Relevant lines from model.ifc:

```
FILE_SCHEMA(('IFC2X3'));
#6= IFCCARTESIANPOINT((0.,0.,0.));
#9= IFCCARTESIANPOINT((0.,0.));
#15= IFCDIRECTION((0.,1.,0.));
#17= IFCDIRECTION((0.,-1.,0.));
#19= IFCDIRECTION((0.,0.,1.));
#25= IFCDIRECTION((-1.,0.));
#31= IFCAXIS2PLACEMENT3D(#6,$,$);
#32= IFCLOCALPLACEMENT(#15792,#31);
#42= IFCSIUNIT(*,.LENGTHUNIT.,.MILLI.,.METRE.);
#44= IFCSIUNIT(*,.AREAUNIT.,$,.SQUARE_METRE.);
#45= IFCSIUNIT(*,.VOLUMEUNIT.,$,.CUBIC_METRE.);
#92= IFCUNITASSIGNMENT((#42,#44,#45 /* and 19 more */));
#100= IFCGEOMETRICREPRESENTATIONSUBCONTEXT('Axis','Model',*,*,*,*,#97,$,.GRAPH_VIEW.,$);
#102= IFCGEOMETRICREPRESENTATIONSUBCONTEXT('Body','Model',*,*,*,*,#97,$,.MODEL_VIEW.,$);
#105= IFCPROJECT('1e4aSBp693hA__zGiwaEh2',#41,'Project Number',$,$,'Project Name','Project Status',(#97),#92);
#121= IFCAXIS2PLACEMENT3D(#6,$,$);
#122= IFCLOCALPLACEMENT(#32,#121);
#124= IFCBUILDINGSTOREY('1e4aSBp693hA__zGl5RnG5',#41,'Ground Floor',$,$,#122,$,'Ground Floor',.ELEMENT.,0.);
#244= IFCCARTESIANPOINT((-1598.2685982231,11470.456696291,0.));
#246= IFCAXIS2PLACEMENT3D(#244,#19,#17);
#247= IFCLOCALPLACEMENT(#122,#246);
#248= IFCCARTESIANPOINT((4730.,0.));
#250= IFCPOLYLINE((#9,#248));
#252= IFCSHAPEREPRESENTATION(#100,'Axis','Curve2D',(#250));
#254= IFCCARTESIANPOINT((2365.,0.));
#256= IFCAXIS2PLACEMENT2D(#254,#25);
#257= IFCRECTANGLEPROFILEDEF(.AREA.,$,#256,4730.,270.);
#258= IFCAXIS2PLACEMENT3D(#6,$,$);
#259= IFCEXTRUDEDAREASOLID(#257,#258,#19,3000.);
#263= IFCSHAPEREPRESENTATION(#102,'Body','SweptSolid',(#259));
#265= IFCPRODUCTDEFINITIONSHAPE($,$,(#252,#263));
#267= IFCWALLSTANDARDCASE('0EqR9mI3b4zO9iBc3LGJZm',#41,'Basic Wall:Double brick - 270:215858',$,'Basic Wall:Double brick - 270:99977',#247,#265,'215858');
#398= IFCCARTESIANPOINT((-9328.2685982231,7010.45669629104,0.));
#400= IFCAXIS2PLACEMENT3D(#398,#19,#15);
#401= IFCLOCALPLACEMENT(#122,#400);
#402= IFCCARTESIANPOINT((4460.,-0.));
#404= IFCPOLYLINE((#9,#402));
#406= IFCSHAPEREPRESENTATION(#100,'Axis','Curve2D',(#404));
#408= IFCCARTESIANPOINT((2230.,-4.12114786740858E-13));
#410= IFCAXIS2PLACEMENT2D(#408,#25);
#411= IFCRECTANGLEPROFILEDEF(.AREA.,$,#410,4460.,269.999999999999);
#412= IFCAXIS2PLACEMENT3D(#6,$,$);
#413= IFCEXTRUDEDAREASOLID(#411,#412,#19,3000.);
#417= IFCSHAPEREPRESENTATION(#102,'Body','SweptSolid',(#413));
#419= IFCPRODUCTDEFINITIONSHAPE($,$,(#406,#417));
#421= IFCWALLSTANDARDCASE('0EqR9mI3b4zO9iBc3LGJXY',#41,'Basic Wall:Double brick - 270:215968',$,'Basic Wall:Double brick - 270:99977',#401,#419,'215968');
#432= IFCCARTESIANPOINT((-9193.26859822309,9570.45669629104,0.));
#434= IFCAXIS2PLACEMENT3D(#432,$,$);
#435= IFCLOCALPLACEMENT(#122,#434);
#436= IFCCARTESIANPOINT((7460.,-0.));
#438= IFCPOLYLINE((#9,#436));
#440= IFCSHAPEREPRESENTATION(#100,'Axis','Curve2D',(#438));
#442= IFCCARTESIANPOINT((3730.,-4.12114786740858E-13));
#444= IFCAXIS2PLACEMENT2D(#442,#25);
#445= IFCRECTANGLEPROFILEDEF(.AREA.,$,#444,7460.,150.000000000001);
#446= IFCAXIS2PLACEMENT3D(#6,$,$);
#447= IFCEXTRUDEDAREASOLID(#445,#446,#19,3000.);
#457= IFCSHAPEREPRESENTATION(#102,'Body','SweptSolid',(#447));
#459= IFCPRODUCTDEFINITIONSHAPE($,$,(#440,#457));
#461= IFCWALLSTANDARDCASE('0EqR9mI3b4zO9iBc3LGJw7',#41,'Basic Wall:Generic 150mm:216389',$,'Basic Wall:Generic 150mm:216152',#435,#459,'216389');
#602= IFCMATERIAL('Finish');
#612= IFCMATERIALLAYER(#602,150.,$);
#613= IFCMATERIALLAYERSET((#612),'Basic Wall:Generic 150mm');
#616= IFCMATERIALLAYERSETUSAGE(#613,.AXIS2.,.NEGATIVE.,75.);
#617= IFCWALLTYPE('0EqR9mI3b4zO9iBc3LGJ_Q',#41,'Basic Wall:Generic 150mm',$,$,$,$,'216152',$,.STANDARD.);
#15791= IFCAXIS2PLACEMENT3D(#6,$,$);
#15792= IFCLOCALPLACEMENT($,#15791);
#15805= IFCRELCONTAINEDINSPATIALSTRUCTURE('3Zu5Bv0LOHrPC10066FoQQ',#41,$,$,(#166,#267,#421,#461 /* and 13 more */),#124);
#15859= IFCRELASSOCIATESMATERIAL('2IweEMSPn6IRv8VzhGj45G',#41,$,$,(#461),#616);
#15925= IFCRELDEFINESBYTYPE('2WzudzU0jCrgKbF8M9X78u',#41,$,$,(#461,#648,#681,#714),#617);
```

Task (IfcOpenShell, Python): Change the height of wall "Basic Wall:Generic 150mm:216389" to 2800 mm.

```python
import ifcopenshell
import ifcopenshell.geom
import ifcopenshell.util.representation
import ifcopenshell.util.shape

model = ifcopenshell.open("model.ifc")
settings = ifcopenshell.geom.settings()


def volume(element):
    """Net volume in cubic metres, openings subtracted."""
    shape = ifcopenshell.geom.create_shape(settings, element)
    return ifcopenshell.util.shape.get_volume(shape.geometry)


wall = model.by_guid("0EqR9mI3b4zO9iBc3LGJw7")
before = volume(wall)

body = ifcopenshell.util.representation.get_representation(wall, "Model", "Body")
solid = body.Items[0]
old_height = solid.Depth
solid.Depth = 2800.0
after = volume(wall)

print(f"height {old_height:g} -> {solid.Depth:g}, volume {before:.3f} -> {after:.3f} m3")

model.write("model_updated.ifc")
```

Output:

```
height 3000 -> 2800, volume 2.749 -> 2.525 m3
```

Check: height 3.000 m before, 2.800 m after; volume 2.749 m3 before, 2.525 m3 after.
